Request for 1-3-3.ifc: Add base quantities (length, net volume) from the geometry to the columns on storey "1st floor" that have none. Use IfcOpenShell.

First a look at what the model holds.

```python
import ifcopenshell
import ifcopenshell.util.element
import ifcopenshell.util.unit

model = ifcopenshell.open("1-3-3.ifc")
print(model.schema)
for unit_type in ("LENGTHUNIT", "AREAUNIT", "VOLUMEUNIT"):
    print(unit_type, ifcopenshell.util.unit.calculate_unit_scale(model, unit_type))
storey = next(s for s in model.by_type("IfcBuildingStorey") if s.Name == "1st floor")
columns = [e for e in ifcopenshell.util.element.get_decomposition(storey) if e.is_a("IfcColumn")]
for e in sorted(columns, key=lambda e: e.id()):
    print(e.id(), e.is_a(), e.Name, list(ifcopenshell.util.element.get_psets(e, qtos_only=True)), sep=" | ")
```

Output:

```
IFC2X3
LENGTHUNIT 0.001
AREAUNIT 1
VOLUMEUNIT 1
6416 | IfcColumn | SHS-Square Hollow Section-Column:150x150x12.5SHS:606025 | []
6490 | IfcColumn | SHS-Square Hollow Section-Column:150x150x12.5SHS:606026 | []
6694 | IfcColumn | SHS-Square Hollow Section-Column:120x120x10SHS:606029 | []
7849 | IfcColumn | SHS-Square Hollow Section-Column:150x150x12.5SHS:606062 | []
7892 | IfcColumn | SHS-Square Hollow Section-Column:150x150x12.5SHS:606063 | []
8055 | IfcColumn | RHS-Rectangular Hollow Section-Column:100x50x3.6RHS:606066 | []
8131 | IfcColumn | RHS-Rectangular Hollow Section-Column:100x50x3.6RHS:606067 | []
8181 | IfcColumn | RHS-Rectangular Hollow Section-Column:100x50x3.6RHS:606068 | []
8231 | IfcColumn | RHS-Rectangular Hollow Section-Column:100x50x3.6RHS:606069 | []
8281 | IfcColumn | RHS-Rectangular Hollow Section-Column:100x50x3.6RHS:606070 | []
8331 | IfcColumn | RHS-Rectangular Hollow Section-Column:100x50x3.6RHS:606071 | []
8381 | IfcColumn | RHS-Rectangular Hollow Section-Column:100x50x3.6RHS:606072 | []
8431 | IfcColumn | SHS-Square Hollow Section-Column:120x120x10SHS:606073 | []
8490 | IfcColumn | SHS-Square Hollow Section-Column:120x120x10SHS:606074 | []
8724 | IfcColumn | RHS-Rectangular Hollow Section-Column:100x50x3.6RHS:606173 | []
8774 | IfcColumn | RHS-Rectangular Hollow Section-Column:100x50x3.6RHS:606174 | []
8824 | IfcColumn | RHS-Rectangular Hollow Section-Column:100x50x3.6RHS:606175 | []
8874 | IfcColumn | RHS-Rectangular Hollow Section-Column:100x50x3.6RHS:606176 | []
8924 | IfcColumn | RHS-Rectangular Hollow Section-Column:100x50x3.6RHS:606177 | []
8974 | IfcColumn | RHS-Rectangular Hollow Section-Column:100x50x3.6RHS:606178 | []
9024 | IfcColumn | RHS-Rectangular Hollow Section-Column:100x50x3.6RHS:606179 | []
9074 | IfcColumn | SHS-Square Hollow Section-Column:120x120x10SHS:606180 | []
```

```python
import ifcopenshell
import ifcopenshell.api.pset
import ifcopenshell.geom
import ifcopenshell.util.element
import ifcopenshell.util.shape
import ifcopenshell.util.unit

model = ifcopenshell.open("1-3-3.ifc")
unit_scale = ifcopenshell.util.unit.calculate_unit_scale(model)
volume_scale = ifcopenshell.util.unit.calculate_unit_scale(model, "VOLUMEUNIT")
settings = ifcopenshell.geom.settings()

storey = next(s for s in model.by_type("IfcBuildingStorey") if s.Name == "1st floor")
columns = [e for e in ifcopenshell.util.element.get_decomposition(storey) if e.is_a("IfcColumn")]

for e in sorted(columns, key=lambda e: e.id()):
    if ifcopenshell.util.element.get_psets(e, qtos_only=True, should_inherit=False):
        continue
    # Geometry comes back in metres, in the element's own axes.
    shape = ifcopenshell.geom.create_shape(settings, e)
    values = {
        "Length": ifcopenshell.util.shape.get_z(shape.geometry) / unit_scale,
        "NetVolume": ifcopenshell.util.shape.get_volume(shape.geometry) / volume_scale,
    }
    qto = ifcopenshell.api.pset.add_qto(model, product=e, name="BaseQuantities")
    ifcopenshell.api.pset.edit_qto(model, qto=qto, properties=values)
    print(e.id(), {k: round(v, 3) for k, v in values.items()})

model.write("1-3-3_rev.ifc")
```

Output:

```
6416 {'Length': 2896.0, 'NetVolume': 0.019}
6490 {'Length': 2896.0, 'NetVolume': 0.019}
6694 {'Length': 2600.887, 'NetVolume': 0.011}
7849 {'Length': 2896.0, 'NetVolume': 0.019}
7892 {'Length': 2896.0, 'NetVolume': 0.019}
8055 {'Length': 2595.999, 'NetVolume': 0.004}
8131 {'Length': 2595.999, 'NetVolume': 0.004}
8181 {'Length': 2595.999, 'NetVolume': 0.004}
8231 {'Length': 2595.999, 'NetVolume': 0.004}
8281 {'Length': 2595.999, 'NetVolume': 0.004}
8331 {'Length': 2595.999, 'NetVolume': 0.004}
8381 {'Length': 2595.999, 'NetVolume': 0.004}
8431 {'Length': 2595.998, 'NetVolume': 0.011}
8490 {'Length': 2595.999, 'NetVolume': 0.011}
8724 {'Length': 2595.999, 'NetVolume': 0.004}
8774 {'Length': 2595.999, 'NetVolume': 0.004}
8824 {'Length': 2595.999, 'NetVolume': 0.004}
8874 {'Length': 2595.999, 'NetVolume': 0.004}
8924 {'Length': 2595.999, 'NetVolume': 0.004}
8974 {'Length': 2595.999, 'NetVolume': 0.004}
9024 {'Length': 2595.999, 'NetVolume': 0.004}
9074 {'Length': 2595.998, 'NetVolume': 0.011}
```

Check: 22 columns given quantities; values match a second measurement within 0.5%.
